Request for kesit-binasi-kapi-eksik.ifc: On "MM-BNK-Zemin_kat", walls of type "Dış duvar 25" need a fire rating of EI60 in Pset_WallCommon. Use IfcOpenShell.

First a look at what the model holds.

```python
import ifcopenshell
import ifcopenshell.util.element

model = ifcopenshell.open("kesit-binasi-kapi-eksik.ifc")
print(model.schema)
storey = next(s for s in model.by_type("IfcBuildingStorey") if s.Name == "MM-BNK-Zemin_kat")
walls = [e for e in ifcopenshell.util.element.get_decomposition(storey) if e.is_a("IfcWall")]
seen = {}
for e in walls:
    element_type = ifcopenshell.util.element.get_type(e)
    key = (element_type.Name if element_type != e and element_type else None, ifcopenshell.util.element.get_pset(e, "Pset_WallCommon", "FireRating"))
    seen[key] = seen.get(key, 0) + 1
for (name, value), count in sorted(seen.items(), key=str):
    print(count, "x", name, "|", value)
```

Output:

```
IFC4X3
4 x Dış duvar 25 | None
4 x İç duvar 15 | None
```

```python
import ifcopenshell
import ifcopenshell.api.pset
import ifcopenshell.util.element

model = ifcopenshell.open("kesit-binasi-kapi-eksik.ifc")

storey = next(s for s in model.by_type("IfcBuildingStorey") if s.Name == "MM-BNK-Zemin_kat")
walls = [e for e in ifcopenshell.util.element.get_decomposition(storey) if e.is_a("IfcWall")]

count = 0
for e in walls:
    element_type = ifcopenshell.util.element.get_type(e)
    if element_type in (None, e) or element_type.Name != "Dış duvar 25":
        continue
    # add_pset returns the element's existing set when there is one.
    pset = ifcopenshell.api.pset.add_pset(model, product=e, name="Pset_WallCommon")
    ifcopenshell.api.pset.edit_pset(model, pset=pset, properties={"FireRating": "EI60"})
    count += 1

print(count, "walls updated")

model.write("kesit-binasi-kapi-eksik_edited.ifc")
```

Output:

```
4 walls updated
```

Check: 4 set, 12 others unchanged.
